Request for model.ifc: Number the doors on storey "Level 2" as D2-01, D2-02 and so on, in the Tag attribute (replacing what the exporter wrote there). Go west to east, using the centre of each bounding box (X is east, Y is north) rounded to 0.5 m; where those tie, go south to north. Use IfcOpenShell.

First a look at what the model holds.

```python
import ifcopenshell
import ifcopenshell.util.element
import ifcopenshell.util.placement

model = ifcopenshell.open("model.ifc")
print(model.schema)
storey = next(s for s in model.by_type("IfcBuildingStorey") if s.Name == "Level 2")
doors = [e for e in ifcopenshell.util.element.get_decomposition(storey) if e.is_a("IfcDoor")]
for e in sorted(doors, key=lambda e: e.id()):
    origin = ifcopenshell.util.placement.get_local_placement(e.ObjectPlacement)[:3, 3]
    print(e.id(), e.Tag, e.Name, origin.round(2) + 0.0, sep=" | ")
```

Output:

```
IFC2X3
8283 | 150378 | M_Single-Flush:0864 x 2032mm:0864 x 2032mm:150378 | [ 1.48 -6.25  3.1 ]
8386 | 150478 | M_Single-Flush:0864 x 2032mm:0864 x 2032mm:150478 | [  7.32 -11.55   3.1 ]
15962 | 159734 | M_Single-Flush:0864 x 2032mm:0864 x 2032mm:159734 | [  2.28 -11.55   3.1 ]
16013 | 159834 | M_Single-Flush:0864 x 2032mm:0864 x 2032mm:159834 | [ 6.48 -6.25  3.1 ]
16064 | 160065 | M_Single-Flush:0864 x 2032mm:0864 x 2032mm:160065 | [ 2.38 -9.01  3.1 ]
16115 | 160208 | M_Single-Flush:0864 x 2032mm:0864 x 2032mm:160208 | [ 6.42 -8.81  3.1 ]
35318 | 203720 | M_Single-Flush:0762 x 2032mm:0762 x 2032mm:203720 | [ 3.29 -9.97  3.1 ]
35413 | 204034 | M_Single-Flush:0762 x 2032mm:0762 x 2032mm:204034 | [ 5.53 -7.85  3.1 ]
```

```python
import ifcopenshell
import ifcopenshell.geom
import ifcopenshell.util.element
import ifcopenshell.util.shape

model = ifcopenshell.open("model.ifc")
settings = ifcopenshell.geom.settings()
settings.set("use-world-coords", True)


def centre(element):
    shape = ifcopenshell.geom.create_shape(settings, element)
    return ifcopenshell.util.shape.get_bbox_centroid(shape.geometry)


storey = next(s for s in model.by_type("IfcBuildingStorey") if s.Name == "Level 2")
doors = [e for e in ifcopenshell.util.element.get_decomposition(storey) if e.is_a("IfcDoor")]

# Insertion points can sit at a corner or the storey origin, so sort by the geometry (in metres).
centres = {e: centre(e) for e in doors}
doors.sort(key=lambda e: (round(centres[e][0] / 0.5), centres[e][1]))

for i, e in enumerate(doors, start=1):
    number = f"D2-{i:02d}"
    e.Tag = number
    print(e.id(), number)

model.write("model_v2.ifc")
```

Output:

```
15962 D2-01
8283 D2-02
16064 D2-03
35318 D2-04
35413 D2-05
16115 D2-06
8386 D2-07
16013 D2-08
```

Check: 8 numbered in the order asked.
